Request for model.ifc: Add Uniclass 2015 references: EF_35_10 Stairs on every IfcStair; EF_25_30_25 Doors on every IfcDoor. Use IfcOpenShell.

First a look at what the model holds.

```python
import ifcopenshell

model = ifcopenshell.open("model.ifc")
print(model.schema)
print("classifications:", [c.Name for c in model.by_type("IfcClassification")])
for ifc_class in ("IfcDoor", "IfcRoof", "IfcStair", "IfcWall", "IfcWindow"):
    print(ifc_class, len(model.by_type(ifc_class)))
```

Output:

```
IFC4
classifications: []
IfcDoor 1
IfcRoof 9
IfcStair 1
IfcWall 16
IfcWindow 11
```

```python
import ifcopenshell
import ifcopenshell.api.classification

model = ifcopenshell.open("model.ifc")

system = ifcopenshell.api.classification.add_classification(model, classification="Uniclass 2015")

codes = {
    "IfcStair": ("EF_35_10", "Stairs"),
    "IfcDoor": ("EF_25_30_25", "Doors"),
}
for ifc_class, (code, name) in codes.items():
    products = model.by_type(ifc_class)
    ifcopenshell.api.classification.add_reference(
        model, products=products, classification=system, identification=code, name=name
    )
    print(code, len(products))

model.write("model_edited.ifc")
```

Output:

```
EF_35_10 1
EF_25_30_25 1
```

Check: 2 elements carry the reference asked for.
